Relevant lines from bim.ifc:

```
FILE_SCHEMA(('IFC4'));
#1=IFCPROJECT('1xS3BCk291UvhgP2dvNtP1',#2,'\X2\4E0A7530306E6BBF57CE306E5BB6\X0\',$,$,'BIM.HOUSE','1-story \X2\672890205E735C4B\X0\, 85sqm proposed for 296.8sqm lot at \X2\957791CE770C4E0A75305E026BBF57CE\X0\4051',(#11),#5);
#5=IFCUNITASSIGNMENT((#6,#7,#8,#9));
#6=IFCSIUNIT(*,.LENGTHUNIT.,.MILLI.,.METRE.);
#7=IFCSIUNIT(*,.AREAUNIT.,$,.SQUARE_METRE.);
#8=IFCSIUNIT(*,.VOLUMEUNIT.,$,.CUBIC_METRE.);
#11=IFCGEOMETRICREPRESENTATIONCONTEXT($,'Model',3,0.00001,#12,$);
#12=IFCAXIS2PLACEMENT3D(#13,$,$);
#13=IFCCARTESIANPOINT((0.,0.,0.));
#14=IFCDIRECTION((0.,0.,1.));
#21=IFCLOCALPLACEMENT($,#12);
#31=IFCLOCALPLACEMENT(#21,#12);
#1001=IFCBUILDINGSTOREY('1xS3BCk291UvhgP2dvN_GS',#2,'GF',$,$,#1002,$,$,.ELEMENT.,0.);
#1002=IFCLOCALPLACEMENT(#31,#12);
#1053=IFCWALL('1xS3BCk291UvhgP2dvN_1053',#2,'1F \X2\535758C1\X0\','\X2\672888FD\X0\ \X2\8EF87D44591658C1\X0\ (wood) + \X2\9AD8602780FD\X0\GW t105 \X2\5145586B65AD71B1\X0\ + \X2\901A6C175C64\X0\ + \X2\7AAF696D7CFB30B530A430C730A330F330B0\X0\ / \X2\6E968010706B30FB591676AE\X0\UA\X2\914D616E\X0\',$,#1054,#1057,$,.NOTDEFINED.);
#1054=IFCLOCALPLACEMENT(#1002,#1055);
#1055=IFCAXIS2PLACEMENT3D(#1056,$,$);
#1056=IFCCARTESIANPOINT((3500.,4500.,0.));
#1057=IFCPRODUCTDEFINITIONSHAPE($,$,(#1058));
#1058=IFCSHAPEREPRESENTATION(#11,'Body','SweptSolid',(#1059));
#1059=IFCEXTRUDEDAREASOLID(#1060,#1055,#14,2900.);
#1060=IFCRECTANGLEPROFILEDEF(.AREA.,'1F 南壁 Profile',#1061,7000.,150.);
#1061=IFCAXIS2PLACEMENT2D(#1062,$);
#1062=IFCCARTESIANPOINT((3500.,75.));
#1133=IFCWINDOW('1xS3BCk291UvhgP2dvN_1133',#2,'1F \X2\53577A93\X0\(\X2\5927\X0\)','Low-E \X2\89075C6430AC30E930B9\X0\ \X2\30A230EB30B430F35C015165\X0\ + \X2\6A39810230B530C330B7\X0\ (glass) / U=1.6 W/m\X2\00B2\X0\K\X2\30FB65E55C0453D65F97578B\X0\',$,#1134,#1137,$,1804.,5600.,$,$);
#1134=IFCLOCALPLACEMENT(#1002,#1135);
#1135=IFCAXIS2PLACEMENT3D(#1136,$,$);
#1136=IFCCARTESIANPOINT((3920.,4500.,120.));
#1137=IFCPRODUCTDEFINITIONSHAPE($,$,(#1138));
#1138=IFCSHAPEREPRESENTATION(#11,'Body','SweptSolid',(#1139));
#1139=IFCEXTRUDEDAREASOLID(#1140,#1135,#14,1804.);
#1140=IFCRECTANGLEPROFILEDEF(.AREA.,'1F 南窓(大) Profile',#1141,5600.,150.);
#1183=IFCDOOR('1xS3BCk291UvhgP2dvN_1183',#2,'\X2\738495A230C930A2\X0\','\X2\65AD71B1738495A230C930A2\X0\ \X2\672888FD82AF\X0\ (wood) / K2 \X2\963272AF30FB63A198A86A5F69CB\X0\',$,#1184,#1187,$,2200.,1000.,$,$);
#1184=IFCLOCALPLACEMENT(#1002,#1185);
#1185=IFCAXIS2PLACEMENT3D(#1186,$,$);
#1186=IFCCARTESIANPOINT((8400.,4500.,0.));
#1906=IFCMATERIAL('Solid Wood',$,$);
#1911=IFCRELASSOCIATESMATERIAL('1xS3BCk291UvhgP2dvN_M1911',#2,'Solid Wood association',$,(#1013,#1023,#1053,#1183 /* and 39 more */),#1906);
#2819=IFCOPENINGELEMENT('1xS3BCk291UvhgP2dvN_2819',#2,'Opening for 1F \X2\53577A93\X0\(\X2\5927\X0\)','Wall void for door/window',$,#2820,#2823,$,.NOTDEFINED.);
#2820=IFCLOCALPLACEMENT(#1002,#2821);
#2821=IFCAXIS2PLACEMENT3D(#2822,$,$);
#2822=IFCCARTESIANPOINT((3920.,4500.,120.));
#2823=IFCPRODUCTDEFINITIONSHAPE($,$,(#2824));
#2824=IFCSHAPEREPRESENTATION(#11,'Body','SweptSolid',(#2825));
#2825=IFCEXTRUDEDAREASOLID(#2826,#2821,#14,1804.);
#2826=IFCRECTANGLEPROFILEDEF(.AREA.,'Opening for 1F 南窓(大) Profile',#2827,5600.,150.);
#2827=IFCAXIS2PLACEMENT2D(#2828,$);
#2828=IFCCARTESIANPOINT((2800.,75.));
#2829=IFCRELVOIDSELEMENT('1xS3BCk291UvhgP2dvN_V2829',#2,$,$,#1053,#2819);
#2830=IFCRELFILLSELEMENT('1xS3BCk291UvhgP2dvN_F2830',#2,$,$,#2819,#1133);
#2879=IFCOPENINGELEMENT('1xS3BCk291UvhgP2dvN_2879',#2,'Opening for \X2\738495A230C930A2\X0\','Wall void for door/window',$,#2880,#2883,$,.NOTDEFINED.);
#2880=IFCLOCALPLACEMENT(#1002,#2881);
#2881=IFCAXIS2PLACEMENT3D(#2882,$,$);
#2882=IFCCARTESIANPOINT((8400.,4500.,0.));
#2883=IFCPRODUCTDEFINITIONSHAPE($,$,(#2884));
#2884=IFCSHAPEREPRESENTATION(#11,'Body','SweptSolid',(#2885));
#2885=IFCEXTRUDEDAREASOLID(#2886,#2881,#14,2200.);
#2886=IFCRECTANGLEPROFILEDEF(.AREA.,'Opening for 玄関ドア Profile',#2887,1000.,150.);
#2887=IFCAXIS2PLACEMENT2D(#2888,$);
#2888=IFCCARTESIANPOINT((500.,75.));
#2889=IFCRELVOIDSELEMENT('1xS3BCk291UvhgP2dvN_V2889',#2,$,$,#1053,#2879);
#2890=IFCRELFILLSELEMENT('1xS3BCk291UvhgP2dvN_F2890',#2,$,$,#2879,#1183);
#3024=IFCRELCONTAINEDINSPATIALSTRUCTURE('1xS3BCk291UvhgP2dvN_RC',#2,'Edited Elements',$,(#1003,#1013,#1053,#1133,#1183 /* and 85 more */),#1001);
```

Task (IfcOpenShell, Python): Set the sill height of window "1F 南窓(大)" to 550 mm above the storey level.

```python
import numpy as np
import ifcopenshell
import ifcopenshell.api.geometry
import ifcopenshell.geom
import ifcopenshell.util.element
import ifcopenshell.util.placement
import ifcopenshell.util.shape
import ifcopenshell.util.unit

model = ifcopenshell.open("bim.ifc")
unit_scale = ifcopenshell.util.unit.calculate_unit_scale(model)

window = model.by_guid("1xS3BCk291UvhgP2dvN_1133")
opening = window.FillsVoids[0].RelatingOpeningElement
storey = ifcopenshell.util.element.get_container(window, ifc_class="IfcBuildingStorey")
level = ifcopenshell.util.placement.get_local_placement(storey.ObjectPlacement)[2, 3]

# The opening's origin need not be at the sill, so measure its lowest point.
shape = ifcopenshell.geom.create_shape(ifcopenshell.geom.settings(), opening)
bottom = ifcopenshell.util.shape.get_shape_bottom_elevation(shape, shape.geometry) / unit_scale
dz = level + 0.55 / unit_scale - bottom

shift = np.array([0.0, 0.0, dz])
# The window is not placed relative to its opening, so move both.
for product in (opening, window):
    matrix = ifcopenshell.util.placement.get_local_placement(product.ObjectPlacement)
    matrix[:3, 3] += shift
    ifcopenshell.api.geometry.edit_object_placement(model, product=product, matrix=matrix, is_si=False)

print(f"moved by {dz * unit_scale:+.3f} m")

model.write("bim_rev.ifc")
```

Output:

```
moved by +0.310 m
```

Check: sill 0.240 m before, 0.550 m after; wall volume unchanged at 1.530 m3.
